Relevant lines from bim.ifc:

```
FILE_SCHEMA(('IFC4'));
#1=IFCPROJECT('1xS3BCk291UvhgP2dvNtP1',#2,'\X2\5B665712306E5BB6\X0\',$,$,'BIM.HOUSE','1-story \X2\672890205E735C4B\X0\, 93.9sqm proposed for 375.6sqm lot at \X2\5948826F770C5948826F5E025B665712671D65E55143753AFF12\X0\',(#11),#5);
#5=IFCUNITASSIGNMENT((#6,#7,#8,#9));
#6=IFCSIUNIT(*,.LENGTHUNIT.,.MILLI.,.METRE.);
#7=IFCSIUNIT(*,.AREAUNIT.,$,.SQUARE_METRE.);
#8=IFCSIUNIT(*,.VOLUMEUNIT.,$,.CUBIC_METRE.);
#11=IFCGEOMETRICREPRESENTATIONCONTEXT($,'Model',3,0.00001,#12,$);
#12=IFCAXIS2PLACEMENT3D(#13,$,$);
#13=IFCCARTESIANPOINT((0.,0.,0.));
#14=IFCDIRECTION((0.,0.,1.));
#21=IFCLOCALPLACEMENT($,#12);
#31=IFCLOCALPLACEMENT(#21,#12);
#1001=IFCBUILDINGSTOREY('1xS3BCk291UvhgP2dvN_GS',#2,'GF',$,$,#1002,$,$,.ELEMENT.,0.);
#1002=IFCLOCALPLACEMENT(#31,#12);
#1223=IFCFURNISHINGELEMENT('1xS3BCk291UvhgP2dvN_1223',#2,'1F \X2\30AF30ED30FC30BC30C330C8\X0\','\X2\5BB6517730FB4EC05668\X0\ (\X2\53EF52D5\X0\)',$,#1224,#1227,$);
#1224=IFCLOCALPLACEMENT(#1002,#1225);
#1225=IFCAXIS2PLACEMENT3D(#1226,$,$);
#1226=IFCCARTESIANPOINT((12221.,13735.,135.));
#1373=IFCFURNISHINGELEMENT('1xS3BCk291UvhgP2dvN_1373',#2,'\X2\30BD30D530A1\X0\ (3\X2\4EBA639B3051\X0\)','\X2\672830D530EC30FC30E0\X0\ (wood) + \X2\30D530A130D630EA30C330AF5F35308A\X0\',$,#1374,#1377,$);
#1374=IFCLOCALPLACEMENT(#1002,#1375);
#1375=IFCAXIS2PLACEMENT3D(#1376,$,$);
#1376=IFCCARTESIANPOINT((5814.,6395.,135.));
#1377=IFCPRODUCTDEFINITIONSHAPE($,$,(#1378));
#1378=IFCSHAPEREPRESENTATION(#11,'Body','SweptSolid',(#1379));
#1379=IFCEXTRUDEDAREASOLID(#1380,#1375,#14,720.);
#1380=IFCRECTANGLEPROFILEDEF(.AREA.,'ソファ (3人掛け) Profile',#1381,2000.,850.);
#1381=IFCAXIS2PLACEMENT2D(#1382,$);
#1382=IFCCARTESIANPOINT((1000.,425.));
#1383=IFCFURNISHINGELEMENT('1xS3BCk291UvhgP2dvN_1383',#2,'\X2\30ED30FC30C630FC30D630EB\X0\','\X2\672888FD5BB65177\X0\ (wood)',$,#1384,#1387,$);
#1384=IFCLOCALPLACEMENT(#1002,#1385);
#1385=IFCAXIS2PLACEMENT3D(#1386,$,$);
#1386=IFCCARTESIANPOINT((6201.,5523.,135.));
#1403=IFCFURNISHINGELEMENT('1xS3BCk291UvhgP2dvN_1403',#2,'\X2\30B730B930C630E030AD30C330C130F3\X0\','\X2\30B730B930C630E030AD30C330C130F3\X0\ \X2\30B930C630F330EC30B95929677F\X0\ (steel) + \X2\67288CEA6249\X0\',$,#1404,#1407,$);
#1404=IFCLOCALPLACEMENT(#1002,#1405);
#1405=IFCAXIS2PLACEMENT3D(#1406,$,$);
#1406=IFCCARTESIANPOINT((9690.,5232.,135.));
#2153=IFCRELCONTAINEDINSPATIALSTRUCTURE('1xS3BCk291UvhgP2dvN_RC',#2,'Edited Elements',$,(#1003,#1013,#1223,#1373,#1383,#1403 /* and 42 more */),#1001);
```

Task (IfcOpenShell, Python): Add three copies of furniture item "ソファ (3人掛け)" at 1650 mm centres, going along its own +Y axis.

```python
import ifcopenshell
import ifcopenshell.api.geometry
import ifcopenshell.api.root
import ifcopenshell.util.element
import ifcopenshell.util.placement

model = ifcopenshell.open("bim.ifc")


def reuse_history(source, copy):
    """copy_class also copies each property set's owner history, people and application; keep the originals."""
    for rel in copy.IsDefinedBy:
        if rel.is_a("IfcRelDefinesByProperties") and (history := rel.RelatingPropertyDefinition.OwnerHistory):
            rel.RelatingPropertyDefinition.OwnerHistory = source.OwnerHistory
            ifcopenshell.util.element.remove_deep2(model, history)


source = model.by_guid("1xS3BCk291UvhgP2dvN_1373")
base = ifcopenshell.util.placement.get_local_placement(source.ObjectPlacement)
step = base[:3, 1] * 1650.0

for i in range(1, 4):
    copy = ifcopenshell.api.root.copy_class(model, product=source)
    copy.Representation = ifcopenshell.util.element.copy_deep(
        model, source.Representation, exclude=["IfcGeometricRepresentationContext", "IfcRepresentationMap"]
    )
    reuse_history(source, copy)
    matrix = base.copy()
    matrix[:3, 3] += i * step
    print("added at", matrix[:3, 3].round(3) + 0.0)
    ifcopenshell.api.geometry.edit_object_placement(model, product=copy, matrix=matrix, is_si=False)

model.write("bim_edited.ifc")
```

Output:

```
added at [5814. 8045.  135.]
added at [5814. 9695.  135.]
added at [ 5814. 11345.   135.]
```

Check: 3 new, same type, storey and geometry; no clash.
